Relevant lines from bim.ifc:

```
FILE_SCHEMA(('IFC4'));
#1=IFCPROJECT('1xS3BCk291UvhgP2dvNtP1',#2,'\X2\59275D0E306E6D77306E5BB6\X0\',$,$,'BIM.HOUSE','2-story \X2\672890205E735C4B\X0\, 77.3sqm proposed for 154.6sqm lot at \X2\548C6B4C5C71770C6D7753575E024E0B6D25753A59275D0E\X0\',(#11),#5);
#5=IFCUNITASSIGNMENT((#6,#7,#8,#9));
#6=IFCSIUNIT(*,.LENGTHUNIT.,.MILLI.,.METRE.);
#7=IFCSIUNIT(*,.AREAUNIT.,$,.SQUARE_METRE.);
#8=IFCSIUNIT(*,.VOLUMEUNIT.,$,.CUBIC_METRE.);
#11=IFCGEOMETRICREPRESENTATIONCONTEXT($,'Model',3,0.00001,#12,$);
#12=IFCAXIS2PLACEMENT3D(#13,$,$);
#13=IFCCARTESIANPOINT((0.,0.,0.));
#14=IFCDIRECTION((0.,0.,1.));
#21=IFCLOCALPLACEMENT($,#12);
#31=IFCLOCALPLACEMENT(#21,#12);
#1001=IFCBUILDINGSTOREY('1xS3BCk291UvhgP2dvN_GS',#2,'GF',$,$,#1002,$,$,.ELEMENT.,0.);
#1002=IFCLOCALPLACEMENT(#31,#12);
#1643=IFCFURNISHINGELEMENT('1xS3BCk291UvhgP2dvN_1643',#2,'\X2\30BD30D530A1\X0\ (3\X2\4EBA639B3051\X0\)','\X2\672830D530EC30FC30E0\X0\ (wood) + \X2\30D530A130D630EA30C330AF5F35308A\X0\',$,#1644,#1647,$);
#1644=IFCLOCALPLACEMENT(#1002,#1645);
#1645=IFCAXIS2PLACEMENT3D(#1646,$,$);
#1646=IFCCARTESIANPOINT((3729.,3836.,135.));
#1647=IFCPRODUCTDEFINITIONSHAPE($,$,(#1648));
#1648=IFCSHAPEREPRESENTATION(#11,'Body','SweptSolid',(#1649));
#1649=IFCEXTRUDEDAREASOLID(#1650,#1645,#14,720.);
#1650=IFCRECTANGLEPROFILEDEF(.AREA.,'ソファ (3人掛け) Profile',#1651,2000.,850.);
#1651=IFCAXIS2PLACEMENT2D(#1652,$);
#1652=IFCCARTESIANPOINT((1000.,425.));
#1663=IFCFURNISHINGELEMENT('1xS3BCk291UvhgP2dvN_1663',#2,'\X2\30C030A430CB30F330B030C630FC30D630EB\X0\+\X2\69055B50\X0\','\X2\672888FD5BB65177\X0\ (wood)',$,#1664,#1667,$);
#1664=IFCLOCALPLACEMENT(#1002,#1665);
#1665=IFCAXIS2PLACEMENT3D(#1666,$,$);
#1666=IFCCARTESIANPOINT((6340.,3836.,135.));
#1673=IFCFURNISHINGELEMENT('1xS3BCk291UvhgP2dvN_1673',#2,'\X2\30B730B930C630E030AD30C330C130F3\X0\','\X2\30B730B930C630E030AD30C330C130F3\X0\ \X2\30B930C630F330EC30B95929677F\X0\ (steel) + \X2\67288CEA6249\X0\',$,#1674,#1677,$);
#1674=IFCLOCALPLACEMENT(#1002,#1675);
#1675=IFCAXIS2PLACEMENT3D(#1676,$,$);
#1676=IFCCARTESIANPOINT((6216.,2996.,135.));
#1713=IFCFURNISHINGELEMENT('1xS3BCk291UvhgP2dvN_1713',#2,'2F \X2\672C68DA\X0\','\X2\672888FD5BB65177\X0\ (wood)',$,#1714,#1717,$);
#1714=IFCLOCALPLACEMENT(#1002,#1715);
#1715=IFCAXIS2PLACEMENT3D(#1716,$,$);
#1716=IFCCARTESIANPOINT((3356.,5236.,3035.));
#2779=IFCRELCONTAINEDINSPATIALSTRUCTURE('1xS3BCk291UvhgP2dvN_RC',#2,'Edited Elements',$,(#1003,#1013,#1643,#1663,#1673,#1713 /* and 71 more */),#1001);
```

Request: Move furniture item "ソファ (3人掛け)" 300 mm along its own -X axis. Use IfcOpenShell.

```python
import ifcopenshell
import ifcopenshell.api.geometry
import ifcopenshell.util.placement
import ifcopenshell.util.unit

model = ifcopenshell.open("bim.ifc")
unit_scale = ifcopenshell.util.unit.calculate_unit_scale(model)

item = model.by_guid("1xS3BCk291UvhgP2dvN_1643")
matrix = ifcopenshell.util.placement.get_local_placement(item.ObjectPlacement)
matrix[:3, 3] -= matrix[:3, 0] * 0.3 / unit_scale
ifcopenshell.api.geometry.edit_object_placement(model, product=item, matrix=matrix, is_si=False)

print(ifcopenshell.util.placement.get_local_placement(item.ObjectPlacement).round(3) + 0.0)

model.write("bim_edited.ifc")
```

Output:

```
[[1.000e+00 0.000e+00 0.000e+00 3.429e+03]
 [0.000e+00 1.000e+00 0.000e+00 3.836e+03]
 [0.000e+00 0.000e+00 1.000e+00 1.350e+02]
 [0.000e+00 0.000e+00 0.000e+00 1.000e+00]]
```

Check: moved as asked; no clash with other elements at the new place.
